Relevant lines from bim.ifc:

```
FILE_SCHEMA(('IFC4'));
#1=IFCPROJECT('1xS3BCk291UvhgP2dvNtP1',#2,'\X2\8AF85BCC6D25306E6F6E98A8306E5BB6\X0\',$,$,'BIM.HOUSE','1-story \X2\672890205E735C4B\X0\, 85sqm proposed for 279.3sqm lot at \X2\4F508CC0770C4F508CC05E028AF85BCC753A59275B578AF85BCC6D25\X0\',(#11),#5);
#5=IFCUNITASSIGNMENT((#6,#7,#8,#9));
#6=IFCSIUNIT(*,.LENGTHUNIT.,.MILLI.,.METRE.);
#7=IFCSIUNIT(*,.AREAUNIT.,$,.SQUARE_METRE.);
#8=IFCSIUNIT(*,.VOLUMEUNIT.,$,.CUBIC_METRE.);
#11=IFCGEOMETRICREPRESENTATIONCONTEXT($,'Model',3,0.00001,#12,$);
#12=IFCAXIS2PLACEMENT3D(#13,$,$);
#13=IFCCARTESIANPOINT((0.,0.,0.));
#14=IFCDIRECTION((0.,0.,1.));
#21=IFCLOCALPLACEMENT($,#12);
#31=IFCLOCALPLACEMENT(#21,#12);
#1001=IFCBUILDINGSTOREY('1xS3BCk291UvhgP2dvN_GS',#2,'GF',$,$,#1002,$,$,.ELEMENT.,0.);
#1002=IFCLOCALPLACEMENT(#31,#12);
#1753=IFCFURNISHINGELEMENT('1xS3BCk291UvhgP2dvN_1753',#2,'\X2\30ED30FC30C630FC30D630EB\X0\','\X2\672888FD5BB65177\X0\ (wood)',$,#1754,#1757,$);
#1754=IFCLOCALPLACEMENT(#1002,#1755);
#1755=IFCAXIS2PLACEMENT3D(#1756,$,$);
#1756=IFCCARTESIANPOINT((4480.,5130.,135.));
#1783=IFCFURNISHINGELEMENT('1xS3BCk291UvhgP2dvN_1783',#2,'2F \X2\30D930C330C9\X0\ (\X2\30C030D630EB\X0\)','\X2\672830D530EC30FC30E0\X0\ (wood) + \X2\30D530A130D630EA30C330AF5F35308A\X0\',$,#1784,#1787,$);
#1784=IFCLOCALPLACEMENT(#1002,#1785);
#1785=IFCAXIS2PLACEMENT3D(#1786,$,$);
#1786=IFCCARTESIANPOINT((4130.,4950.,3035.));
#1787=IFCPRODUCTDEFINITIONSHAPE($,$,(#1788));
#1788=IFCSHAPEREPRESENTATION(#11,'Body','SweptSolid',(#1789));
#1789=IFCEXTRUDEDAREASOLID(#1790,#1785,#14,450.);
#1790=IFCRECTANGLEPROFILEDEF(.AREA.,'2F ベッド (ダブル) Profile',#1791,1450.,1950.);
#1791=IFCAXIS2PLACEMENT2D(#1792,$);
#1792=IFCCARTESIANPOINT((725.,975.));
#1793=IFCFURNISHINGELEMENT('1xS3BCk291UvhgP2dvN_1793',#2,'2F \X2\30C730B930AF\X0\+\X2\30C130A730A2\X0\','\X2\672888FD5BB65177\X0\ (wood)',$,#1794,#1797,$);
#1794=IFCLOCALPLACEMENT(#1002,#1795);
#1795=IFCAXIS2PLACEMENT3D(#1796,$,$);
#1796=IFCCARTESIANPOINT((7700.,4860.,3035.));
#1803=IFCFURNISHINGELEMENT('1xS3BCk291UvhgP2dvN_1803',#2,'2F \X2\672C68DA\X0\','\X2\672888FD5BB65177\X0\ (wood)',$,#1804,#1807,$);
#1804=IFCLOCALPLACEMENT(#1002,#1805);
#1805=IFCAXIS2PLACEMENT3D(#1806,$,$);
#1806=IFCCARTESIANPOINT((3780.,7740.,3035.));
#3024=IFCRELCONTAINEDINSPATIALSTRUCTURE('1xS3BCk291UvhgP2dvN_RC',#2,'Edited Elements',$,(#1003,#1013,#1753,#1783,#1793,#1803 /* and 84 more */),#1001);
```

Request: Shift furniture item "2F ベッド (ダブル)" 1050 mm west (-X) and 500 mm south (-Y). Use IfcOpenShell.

```python
import ifcopenshell
import ifcopenshell.api.geometry
import ifcopenshell.util.placement
import ifcopenshell.util.unit

model = ifcopenshell.open("bim.ifc")
unit_scale = ifcopenshell.util.unit.calculate_unit_scale(model)

item = model.by_guid("1xS3BCk291UvhgP2dvN_1783")
matrix = ifcopenshell.util.placement.get_local_placement(item.ObjectPlacement)
matrix[0, 3] -= 1.05 / unit_scale
matrix[1, 3] -= 0.5 / unit_scale
ifcopenshell.api.geometry.edit_object_placement(model, product=item, matrix=matrix, is_si=False)

print(ifcopenshell.util.placement.get_local_placement(item.ObjectPlacement).round(3) + 0.0)

model.write("bim_updated.ifc")
```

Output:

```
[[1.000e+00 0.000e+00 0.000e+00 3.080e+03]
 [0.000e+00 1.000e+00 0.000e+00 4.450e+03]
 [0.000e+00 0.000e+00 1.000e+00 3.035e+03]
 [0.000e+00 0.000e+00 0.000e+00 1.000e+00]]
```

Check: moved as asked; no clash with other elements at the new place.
